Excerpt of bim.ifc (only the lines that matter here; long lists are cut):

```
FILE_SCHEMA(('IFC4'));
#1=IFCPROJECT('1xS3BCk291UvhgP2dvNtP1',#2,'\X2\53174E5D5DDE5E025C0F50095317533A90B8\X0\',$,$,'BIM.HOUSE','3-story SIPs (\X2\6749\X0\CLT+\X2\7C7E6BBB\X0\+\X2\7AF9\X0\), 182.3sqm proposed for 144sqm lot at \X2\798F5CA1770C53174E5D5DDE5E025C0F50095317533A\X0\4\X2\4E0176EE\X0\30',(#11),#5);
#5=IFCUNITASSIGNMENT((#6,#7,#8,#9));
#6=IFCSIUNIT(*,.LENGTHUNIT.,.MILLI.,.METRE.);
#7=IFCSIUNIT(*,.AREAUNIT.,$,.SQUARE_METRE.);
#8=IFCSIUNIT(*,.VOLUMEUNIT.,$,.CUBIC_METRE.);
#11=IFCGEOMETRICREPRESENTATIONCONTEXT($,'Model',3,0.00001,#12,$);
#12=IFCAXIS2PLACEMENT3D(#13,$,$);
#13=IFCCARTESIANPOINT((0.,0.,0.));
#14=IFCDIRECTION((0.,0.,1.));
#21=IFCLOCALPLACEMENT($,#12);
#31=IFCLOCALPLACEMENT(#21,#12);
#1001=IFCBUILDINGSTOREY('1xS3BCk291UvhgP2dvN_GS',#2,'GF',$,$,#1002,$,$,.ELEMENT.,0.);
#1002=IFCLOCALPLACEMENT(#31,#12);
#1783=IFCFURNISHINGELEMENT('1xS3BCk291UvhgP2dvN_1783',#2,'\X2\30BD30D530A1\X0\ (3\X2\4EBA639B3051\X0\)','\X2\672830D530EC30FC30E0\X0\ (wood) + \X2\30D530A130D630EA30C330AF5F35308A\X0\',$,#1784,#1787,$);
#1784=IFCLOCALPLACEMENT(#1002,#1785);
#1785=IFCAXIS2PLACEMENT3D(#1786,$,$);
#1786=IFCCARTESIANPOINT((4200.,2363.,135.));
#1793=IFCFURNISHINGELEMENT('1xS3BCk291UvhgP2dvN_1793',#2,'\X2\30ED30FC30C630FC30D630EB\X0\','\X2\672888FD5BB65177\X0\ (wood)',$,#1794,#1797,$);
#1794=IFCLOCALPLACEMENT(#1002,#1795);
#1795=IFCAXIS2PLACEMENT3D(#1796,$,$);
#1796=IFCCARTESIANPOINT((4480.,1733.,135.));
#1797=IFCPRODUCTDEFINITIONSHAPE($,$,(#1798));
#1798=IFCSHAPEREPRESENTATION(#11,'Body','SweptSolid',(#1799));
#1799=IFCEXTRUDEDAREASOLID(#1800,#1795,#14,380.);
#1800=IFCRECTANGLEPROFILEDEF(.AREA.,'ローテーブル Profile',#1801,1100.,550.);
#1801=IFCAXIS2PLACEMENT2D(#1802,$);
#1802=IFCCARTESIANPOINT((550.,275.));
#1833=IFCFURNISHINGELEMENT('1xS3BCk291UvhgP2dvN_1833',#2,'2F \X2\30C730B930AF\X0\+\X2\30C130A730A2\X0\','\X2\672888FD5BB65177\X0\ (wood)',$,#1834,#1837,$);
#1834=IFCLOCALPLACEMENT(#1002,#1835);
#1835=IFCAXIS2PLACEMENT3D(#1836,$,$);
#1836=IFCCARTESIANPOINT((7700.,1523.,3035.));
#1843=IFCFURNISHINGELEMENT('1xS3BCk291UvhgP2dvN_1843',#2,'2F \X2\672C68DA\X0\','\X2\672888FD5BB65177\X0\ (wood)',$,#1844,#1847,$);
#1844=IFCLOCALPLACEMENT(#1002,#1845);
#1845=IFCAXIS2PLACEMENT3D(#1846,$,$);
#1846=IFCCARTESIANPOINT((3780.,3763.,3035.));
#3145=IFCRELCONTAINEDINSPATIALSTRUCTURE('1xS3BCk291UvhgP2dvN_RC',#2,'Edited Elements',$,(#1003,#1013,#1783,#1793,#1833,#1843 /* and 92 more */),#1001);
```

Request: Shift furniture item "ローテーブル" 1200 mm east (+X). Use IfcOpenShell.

```python
import ifcopenshell
import ifcopenshell.api.geometry
import ifcopenshell.util.placement

model = ifcopenshell.open("bim.ifc")

item = model.by_guid("1xS3BCk291UvhgP2dvN_1793")
matrix = ifcopenshell.util.placement.get_local_placement(item.ObjectPlacement)
matrix[0, 3] += 1200.0
ifcopenshell.api.geometry.edit_object_placement(model, product=item, matrix=matrix, is_si=False)

print(ifcopenshell.util.placement.get_local_placement(item.ObjectPlacement).round(3) + 0.0)

model.write("bim_edited.ifc")
```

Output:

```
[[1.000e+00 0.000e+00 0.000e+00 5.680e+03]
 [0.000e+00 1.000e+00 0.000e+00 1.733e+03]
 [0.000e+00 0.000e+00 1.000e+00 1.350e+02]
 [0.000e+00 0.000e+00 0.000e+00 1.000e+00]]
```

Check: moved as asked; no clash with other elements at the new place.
